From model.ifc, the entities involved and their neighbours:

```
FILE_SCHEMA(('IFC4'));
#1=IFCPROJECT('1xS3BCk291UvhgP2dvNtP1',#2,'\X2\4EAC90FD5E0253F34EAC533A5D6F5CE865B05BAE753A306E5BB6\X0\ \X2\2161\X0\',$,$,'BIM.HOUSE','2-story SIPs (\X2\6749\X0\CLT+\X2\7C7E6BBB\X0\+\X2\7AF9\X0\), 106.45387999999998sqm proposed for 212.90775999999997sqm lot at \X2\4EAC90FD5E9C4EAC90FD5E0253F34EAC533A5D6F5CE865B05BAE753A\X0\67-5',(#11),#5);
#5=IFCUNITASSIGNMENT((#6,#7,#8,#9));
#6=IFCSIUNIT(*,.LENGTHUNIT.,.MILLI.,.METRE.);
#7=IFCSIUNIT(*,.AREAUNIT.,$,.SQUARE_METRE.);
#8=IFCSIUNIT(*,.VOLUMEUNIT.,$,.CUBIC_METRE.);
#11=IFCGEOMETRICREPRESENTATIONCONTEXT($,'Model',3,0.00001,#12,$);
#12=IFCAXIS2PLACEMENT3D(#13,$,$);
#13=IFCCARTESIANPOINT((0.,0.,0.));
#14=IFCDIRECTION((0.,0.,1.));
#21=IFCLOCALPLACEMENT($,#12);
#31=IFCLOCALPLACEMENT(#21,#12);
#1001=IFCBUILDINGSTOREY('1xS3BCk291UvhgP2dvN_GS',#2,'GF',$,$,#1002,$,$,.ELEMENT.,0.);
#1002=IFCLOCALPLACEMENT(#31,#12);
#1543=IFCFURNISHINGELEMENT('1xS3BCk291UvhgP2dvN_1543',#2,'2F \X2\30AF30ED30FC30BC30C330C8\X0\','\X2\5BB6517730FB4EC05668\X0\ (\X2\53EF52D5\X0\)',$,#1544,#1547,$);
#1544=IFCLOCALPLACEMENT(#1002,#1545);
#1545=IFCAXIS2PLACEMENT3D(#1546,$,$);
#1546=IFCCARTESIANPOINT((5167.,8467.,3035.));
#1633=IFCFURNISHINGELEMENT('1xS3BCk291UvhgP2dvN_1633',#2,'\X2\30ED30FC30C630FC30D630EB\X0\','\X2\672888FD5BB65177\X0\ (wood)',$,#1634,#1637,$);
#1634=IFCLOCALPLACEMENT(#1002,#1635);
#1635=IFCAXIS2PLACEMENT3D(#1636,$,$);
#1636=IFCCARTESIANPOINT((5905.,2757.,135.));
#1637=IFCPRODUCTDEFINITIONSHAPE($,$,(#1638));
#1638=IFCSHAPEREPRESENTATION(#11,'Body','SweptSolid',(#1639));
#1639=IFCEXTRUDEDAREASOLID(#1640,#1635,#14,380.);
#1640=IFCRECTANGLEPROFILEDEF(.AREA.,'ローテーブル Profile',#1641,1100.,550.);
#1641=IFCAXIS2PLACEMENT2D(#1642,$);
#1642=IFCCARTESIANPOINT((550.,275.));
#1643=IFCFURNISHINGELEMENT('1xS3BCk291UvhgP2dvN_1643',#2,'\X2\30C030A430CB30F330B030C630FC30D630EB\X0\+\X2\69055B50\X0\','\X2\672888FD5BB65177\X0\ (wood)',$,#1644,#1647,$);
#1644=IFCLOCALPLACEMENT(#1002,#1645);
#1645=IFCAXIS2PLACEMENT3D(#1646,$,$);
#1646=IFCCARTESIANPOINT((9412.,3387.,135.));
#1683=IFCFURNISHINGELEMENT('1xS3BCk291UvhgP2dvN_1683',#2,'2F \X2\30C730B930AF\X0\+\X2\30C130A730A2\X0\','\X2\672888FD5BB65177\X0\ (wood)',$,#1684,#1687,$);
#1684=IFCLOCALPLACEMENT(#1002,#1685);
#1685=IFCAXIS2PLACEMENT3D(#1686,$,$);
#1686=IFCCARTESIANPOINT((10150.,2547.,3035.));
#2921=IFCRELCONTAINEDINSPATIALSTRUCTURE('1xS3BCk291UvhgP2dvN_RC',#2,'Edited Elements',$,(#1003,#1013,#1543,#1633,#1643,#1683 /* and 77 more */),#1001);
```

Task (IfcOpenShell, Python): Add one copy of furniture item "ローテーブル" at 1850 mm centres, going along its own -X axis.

```python
import ifcopenshell
import ifcopenshell.api.geometry
import ifcopenshell.api.root
import ifcopenshell.util.element
import ifcopenshell.util.placement
import ifcopenshell.util.unit

model = ifcopenshell.open("model.ifc")
unit_scale = ifcopenshell.util.unit.calculate_unit_scale(model)


def reuse_history(source, copy):
    """copy_class also copies each property set's owner history, people and application; keep the originals."""
    for rel in copy.IsDefinedBy:
        if rel.is_a("IfcRelDefinesByProperties") and (history := rel.RelatingPropertyDefinition.OwnerHistory):
            rel.RelatingPropertyDefinition.OwnerHistory = source.OwnerHistory
            ifcopenshell.util.element.remove_deep2(model, history)


source = model.by_guid("1xS3BCk291UvhgP2dvN_1633")
base = ifcopenshell.util.placement.get_local_placement(source.ObjectPlacement)
step = -base[:3, 0] * 1.85 / unit_scale

for i in range(1, 2):
    copy = ifcopenshell.api.root.copy_class(model, product=source)
    copy.Representation = ifcopenshell.util.element.copy_deep(
        model, source.Representation, exclude=["IfcGeometricRepresentationContext", "IfcRepresentationMap"]
    )
    reuse_history(source, copy)
    matrix = base.copy()
    matrix[:3, 3] += i * step
    print("added at", matrix[:3, 3].round(3) + 0.0)
    ifcopenshell.api.geometry.edit_object_placement(model, product=copy, matrix=matrix, is_si=False)

model.write("model_rev.ifc")
```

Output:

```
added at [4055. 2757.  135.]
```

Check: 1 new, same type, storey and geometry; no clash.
